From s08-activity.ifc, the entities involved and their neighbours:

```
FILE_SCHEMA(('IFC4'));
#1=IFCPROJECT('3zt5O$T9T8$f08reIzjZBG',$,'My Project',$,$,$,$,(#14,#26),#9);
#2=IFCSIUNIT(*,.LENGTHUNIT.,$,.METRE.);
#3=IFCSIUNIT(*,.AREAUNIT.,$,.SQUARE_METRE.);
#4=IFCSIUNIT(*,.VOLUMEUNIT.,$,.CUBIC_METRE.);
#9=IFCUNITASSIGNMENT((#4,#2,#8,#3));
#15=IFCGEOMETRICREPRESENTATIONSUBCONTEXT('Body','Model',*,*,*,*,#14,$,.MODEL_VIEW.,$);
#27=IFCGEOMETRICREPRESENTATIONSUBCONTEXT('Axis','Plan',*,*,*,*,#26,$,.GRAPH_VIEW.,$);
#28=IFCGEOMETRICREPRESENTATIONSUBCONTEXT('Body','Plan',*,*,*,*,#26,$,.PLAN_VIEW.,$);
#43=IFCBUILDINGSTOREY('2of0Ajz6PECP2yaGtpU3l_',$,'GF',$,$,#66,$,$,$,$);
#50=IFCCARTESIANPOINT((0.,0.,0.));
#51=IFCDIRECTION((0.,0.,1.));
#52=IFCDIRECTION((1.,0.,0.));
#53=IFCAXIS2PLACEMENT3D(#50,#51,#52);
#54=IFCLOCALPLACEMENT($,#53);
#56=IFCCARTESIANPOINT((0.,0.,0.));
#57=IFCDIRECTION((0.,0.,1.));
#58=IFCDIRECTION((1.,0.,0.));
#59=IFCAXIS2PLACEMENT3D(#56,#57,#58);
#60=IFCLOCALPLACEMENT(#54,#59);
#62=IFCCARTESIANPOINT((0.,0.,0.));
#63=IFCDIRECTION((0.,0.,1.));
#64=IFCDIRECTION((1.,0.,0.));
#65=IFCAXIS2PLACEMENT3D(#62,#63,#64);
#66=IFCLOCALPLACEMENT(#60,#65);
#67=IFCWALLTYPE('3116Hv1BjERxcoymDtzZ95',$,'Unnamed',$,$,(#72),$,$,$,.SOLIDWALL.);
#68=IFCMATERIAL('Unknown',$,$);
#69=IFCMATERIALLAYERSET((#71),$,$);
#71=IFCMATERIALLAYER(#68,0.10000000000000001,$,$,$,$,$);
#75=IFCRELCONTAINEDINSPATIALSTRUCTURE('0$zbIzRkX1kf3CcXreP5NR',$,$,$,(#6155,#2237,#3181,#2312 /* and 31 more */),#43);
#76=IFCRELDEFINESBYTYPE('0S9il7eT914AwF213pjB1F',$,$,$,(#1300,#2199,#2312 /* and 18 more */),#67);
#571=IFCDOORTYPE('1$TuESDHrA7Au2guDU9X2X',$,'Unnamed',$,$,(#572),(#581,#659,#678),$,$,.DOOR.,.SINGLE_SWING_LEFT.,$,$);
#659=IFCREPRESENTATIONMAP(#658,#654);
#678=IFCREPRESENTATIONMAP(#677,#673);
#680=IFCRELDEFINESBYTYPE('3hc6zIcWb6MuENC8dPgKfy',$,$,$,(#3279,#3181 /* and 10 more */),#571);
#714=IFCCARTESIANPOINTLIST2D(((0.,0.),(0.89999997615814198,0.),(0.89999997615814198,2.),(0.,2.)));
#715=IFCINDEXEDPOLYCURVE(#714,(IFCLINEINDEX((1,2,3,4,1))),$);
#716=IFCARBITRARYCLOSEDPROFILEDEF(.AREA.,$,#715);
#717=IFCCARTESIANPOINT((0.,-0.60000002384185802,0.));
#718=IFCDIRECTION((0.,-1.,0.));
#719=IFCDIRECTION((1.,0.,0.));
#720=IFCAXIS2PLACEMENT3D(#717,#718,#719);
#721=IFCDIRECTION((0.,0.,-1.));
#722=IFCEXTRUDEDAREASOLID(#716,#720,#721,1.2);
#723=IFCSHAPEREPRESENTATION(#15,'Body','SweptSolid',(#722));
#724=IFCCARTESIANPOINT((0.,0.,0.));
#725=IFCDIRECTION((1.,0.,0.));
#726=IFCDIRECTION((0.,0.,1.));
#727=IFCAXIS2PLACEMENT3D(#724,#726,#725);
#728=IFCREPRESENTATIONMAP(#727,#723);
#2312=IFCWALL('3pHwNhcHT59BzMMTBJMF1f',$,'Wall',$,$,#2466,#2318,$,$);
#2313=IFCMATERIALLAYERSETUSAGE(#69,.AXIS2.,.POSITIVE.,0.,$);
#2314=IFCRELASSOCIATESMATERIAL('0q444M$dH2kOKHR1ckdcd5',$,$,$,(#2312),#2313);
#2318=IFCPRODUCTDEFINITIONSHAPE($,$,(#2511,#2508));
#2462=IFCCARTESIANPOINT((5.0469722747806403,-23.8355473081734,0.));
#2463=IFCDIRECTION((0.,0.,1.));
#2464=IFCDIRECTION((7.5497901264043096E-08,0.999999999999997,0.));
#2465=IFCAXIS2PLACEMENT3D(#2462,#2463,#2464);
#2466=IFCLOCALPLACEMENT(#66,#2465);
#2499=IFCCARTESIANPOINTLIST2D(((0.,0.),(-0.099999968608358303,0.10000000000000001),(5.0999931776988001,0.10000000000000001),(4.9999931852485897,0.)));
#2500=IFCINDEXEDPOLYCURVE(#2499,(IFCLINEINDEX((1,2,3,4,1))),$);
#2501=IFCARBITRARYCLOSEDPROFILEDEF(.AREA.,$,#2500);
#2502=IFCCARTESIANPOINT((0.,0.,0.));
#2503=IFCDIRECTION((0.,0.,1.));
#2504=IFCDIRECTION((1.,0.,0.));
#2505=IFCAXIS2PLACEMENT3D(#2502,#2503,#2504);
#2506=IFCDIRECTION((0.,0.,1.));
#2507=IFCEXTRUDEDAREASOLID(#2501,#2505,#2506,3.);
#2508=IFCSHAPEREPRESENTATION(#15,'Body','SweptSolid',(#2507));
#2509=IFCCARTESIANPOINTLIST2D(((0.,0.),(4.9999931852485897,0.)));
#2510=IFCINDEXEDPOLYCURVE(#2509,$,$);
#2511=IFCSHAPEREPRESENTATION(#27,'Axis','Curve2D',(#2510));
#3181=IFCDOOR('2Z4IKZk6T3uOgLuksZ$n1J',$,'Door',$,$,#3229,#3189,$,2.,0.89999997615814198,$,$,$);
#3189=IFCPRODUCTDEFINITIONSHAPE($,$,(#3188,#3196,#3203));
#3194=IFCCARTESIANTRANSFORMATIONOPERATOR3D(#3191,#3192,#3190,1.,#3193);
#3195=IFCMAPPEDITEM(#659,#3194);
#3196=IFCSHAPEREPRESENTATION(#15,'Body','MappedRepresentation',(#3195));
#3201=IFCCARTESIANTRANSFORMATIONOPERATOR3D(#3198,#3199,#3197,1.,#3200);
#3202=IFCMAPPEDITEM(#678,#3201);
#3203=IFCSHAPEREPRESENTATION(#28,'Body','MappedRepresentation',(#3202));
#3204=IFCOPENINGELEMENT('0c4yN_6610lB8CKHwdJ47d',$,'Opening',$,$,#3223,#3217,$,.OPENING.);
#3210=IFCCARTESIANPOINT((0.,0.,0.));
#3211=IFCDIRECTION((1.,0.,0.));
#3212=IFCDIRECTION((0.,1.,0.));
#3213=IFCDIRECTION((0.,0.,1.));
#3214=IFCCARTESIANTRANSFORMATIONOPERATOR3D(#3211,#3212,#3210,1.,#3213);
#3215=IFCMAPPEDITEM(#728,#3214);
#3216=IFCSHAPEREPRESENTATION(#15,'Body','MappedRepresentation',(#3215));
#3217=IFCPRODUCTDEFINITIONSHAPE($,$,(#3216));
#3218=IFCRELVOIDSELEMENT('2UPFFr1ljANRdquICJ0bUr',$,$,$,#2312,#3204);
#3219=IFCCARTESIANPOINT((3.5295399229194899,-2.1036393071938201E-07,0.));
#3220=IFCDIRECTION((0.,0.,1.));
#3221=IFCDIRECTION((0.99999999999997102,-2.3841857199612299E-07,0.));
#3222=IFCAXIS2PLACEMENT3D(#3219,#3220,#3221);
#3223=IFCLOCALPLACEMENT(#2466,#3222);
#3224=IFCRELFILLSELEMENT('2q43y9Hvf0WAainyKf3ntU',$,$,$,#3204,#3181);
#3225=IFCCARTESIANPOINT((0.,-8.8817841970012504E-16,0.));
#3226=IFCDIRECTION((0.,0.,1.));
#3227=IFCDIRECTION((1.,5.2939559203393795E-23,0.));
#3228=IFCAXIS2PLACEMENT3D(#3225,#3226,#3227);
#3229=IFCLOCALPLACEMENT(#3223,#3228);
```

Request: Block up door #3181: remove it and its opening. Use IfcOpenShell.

```python
import ifcopenshell
import ifcopenshell.api.feature
import ifcopenshell.api.root
import ifcopenshell.geom
import ifcopenshell.util.shape

model = ifcopenshell.open("s08-activity.ifc")
settings = ifcopenshell.geom.settings()


def volume(element):
    """Net volume in cubic metres, openings subtracted."""
    shape = ifcopenshell.geom.create_shape(settings, element)
    return ifcopenshell.util.shape.get_volume(shape.geometry)


door = model.by_id(3181)
opening = door.FillsVoids[0].RelatingOpeningElement
wall = opening.VoidsElements[0].RelatingBuildingElement
before = volume(wall)

ifcopenshell.api.root.remove_product(model, product=door)
ifcopenshell.api.feature.remove_feature(model, feature=opening)

after = volume(wall)

print(f"wall volume {before:.3f} -> {after:.3f} m3")

model.write("s08-activity_updated.ifc")
```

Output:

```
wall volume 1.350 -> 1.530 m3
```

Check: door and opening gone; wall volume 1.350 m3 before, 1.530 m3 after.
